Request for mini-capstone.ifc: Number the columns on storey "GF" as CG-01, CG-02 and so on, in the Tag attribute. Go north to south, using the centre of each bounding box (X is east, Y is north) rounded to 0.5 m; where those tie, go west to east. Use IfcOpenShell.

First a look at what the model holds.

```python
import ifcopenshell
import ifcopenshell.util.element
import ifcopenshell.util.placement

model = ifcopenshell.open("mini-capstone.ifc")
print(model.schema)
storey = next(s for s in model.by_type("IfcBuildingStorey") if s.Name == "GF")
columns = [e for e in ifcopenshell.util.element.get_decomposition(storey) if e.is_a("IfcColumn")]
for e in sorted(columns, key=lambda e: e.id()):
    origin = ifcopenshell.util.placement.get_local_placement(e.ObjectPlacement)[:3, 3]
    print(e.id(), e.Tag, e.Name, origin.round(2) + 0.0, sep=" | ")
```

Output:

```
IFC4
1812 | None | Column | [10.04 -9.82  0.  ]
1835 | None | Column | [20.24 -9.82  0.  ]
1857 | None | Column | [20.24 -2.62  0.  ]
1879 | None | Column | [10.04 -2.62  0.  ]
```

```python
import ifcopenshell
import ifcopenshell.geom
import ifcopenshell.util.element
import ifcopenshell.util.shape

model = ifcopenshell.open("mini-capstone.ifc")
settings = ifcopenshell.geom.settings()
settings.set("use-world-coords", True)


def centre(element):
    shape = ifcopenshell.geom.create_shape(settings, element)
    return ifcopenshell.util.shape.get_bbox_centroid(shape.geometry)


storey = next(s for s in model.by_type("IfcBuildingStorey") if s.Name == "GF")
columns = [e for e in ifcopenshell.util.element.get_decomposition(storey) if e.is_a("IfcColumn")]

# Insertion points can sit at a corner or the storey origin, so sort by the geometry (in metres).
centres = {e: centre(e) for e in columns}
columns.sort(key=lambda e: (-round(centres[e][1] / 0.5), centres[e][0]))

for i, e in enumerate(columns, start=1):
    number = f"CG-{i:02d}"
    e.Tag = number
    print(e.id(), number)

model.write("mini-capstone_edited.ifc")
```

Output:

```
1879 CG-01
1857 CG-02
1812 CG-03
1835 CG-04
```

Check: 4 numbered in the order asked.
